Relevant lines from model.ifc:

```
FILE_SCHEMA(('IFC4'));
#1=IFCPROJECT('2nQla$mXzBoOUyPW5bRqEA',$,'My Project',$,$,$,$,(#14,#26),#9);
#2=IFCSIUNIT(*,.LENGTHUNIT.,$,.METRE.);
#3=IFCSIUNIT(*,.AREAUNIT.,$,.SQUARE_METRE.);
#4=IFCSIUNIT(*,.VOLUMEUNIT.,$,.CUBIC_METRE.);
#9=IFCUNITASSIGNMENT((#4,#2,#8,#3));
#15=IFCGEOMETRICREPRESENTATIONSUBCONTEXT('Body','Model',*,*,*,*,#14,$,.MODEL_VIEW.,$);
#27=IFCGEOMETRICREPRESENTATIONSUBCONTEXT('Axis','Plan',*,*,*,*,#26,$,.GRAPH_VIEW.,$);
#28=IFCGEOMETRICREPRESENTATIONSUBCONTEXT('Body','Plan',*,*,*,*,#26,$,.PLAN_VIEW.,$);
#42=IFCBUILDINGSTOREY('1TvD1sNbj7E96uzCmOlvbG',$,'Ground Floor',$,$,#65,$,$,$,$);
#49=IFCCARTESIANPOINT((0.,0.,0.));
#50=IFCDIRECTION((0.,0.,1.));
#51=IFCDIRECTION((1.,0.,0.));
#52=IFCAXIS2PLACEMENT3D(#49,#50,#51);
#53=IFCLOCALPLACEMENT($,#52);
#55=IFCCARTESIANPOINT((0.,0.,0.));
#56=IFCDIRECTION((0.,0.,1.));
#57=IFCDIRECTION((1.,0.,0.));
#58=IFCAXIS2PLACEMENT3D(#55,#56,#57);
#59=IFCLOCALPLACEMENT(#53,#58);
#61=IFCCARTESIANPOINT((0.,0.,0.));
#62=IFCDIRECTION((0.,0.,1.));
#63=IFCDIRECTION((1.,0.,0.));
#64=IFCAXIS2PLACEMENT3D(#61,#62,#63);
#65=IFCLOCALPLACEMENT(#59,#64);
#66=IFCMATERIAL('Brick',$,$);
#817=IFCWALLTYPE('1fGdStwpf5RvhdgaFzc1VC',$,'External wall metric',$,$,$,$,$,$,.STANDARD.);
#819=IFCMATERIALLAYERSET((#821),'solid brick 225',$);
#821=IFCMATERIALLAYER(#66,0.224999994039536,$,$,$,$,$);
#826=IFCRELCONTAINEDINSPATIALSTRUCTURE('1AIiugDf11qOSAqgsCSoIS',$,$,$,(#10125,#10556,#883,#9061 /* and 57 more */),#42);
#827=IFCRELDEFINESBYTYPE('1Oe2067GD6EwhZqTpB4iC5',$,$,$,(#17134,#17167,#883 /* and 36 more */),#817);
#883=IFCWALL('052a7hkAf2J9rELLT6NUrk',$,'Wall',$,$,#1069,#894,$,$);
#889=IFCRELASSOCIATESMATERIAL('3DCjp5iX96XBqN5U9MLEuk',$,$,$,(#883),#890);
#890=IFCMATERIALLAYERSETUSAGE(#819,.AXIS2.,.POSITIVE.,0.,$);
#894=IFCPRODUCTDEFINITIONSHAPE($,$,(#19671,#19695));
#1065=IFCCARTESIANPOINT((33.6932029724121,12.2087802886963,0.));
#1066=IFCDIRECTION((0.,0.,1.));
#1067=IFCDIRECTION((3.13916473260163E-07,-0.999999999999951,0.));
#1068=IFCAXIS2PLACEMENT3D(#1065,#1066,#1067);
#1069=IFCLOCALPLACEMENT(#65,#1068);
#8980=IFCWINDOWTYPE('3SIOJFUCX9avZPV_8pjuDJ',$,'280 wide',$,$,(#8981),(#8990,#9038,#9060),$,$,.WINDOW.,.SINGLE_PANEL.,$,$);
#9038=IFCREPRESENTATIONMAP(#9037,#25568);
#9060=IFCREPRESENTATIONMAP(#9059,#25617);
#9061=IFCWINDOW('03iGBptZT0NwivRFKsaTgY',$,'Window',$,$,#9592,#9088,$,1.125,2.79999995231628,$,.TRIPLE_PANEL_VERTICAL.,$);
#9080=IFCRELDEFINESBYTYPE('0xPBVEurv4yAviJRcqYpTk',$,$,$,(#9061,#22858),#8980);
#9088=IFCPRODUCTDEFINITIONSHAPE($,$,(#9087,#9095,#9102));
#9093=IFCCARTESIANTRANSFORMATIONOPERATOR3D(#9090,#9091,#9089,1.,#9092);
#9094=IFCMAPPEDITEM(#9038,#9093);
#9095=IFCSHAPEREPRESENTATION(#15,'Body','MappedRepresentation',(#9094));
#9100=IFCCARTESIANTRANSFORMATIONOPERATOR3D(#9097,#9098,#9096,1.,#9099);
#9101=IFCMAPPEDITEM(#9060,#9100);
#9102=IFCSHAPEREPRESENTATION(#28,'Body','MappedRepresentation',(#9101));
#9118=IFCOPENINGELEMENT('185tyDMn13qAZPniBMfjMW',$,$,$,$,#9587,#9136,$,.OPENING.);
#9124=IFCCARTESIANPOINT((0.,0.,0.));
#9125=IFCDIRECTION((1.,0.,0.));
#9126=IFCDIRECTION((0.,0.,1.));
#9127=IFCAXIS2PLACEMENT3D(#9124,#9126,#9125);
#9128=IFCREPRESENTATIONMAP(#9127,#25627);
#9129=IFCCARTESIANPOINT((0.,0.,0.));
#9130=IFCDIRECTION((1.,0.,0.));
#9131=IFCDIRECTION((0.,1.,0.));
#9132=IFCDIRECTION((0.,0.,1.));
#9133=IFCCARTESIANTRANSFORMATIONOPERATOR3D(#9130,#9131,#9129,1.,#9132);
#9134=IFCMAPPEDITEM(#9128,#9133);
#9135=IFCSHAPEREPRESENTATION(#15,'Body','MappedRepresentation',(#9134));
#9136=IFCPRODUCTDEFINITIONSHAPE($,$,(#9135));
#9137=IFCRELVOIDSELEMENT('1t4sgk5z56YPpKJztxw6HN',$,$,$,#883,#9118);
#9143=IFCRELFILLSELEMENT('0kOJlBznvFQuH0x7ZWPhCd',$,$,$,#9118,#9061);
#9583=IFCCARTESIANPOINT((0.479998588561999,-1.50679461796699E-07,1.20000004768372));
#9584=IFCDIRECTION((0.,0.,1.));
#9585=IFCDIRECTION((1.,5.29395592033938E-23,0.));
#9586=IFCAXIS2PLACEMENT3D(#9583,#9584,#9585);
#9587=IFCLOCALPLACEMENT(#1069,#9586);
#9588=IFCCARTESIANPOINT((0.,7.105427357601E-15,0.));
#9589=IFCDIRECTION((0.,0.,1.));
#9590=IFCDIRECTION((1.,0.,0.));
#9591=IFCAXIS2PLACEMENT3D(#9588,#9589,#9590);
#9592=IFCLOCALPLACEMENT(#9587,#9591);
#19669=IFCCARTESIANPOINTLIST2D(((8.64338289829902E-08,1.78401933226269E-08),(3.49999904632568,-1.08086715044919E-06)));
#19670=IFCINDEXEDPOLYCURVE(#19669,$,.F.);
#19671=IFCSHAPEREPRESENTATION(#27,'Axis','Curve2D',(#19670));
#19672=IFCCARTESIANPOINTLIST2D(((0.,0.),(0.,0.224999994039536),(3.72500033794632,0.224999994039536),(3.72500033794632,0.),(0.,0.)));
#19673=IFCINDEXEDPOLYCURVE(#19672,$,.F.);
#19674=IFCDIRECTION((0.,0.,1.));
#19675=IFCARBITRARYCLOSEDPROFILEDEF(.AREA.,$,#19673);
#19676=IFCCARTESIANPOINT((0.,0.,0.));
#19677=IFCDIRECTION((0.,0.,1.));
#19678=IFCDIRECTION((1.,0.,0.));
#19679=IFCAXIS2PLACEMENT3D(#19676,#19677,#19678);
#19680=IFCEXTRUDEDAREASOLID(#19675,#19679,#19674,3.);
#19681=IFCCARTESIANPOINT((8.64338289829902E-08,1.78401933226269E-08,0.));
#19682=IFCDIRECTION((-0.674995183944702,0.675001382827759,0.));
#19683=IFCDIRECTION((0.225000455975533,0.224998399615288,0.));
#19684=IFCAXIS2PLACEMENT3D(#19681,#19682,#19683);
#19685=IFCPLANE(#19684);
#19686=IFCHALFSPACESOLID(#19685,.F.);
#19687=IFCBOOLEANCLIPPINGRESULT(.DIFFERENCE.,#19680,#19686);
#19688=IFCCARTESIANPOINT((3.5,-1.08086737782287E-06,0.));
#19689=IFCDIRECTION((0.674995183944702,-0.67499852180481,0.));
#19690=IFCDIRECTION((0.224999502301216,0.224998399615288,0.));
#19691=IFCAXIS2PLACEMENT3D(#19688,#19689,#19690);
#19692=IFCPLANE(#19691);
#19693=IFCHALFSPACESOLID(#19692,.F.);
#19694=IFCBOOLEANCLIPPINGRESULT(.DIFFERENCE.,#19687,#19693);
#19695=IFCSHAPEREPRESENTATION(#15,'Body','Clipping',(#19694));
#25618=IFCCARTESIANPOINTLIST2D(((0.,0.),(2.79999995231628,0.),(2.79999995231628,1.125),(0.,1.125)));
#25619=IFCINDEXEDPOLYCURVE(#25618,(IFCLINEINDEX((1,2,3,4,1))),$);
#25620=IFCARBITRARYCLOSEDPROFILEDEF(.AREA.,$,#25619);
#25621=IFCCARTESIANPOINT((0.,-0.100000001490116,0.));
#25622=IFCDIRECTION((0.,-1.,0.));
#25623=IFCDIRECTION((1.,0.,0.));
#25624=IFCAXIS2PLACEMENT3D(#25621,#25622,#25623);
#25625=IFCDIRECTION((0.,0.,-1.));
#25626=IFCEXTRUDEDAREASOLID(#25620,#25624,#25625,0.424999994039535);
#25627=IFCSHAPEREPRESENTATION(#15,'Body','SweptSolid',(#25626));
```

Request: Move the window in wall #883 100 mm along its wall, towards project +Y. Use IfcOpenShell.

```python
import ifcopenshell
import ifcopenshell.api.geometry
import ifcopenshell.util.placement

model = ifcopenshell.open("model.ifc")

window = model.by_guid("03iGBptZT0NwivRFKsaTgY")
opening = window.FillsVoids[0].RelatingOpeningElement
wall = opening.VoidsElements[0].RelatingBuildingElement

wall_matrix = ifcopenshell.util.placement.get_local_placement(wall.ObjectPlacement)
shift = wall_matrix[:3, 0] * -0.1
before = ifcopenshell.util.placement.get_local_placement(window.ObjectPlacement)[:3, 3].copy()

# The window is placed relative to its opening, so it follows when the opening moves.
matrix = ifcopenshell.util.placement.get_local_placement(opening.ObjectPlacement)
matrix[:3, 3] += shift
ifcopenshell.api.geometry.edit_object_placement(
    model, product=opening, matrix=matrix, is_si=False, should_transform_children=True
)

after = ifcopenshell.util.placement.get_local_placement(window.ObjectPlacement)[:3, 3]
print("window moved by", (after - before).round(3) + 0.0)

model.write("model-out.ifc")
```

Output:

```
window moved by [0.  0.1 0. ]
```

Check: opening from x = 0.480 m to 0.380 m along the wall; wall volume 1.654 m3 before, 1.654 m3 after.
